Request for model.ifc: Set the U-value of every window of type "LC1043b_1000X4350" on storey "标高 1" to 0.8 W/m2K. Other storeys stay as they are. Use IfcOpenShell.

First a look at what the model holds.

```python
import ifcopenshell
import ifcopenshell.util.element

model = ifcopenshell.open("model.ifc")
print(model.schema)
storey = next(s for s in model.by_type("IfcBuildingStorey") if s.Name == "标高 1")
windows = [e for e in ifcopenshell.util.element.get_decomposition(storey) if e.is_a("IfcWindow")]
seen = {}
for e in windows:
    element_type = ifcopenshell.util.element.get_type(e)
    key = (element_type.Name if element_type != e and element_type else None, ifcopenshell.util.element.get_pset(e, "Pset_WindowCommon", "ThermalTransmittance"))
    seen[key] = seen.get(key, 0) + 1
for (name, value), count in sorted(seen.items(), key=str):
    print(count, "x", name, "|", value)
```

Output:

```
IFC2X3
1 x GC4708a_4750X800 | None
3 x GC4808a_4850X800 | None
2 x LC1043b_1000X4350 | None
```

```python
import ifcopenshell
import ifcopenshell.api.pset
import ifcopenshell.util.element

model = ifcopenshell.open("model.ifc")

storey = next(s for s in model.by_type("IfcBuildingStorey") if s.Name == "标高 1")
windows = [e for e in ifcopenshell.util.element.get_decomposition(storey) if e.is_a("IfcWindow")]

count = 0
for e in windows:
    element_type = ifcopenshell.util.element.get_type(e)
    if element_type in (None, e) or element_type.Name != "LC1043b_1000X4350":
        continue
    # add_pset returns the element's existing set when there is one.
    pset = ifcopenshell.api.pset.add_pset(model, product=e, name="Pset_WindowCommon")
    ifcopenshell.api.pset.edit_pset(model, pset=pset, properties={"ThermalTransmittance": 0.8})
    count += 1

print(count, "windows updated")

model.write("model_v2.ifc")
```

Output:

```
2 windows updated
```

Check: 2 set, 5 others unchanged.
